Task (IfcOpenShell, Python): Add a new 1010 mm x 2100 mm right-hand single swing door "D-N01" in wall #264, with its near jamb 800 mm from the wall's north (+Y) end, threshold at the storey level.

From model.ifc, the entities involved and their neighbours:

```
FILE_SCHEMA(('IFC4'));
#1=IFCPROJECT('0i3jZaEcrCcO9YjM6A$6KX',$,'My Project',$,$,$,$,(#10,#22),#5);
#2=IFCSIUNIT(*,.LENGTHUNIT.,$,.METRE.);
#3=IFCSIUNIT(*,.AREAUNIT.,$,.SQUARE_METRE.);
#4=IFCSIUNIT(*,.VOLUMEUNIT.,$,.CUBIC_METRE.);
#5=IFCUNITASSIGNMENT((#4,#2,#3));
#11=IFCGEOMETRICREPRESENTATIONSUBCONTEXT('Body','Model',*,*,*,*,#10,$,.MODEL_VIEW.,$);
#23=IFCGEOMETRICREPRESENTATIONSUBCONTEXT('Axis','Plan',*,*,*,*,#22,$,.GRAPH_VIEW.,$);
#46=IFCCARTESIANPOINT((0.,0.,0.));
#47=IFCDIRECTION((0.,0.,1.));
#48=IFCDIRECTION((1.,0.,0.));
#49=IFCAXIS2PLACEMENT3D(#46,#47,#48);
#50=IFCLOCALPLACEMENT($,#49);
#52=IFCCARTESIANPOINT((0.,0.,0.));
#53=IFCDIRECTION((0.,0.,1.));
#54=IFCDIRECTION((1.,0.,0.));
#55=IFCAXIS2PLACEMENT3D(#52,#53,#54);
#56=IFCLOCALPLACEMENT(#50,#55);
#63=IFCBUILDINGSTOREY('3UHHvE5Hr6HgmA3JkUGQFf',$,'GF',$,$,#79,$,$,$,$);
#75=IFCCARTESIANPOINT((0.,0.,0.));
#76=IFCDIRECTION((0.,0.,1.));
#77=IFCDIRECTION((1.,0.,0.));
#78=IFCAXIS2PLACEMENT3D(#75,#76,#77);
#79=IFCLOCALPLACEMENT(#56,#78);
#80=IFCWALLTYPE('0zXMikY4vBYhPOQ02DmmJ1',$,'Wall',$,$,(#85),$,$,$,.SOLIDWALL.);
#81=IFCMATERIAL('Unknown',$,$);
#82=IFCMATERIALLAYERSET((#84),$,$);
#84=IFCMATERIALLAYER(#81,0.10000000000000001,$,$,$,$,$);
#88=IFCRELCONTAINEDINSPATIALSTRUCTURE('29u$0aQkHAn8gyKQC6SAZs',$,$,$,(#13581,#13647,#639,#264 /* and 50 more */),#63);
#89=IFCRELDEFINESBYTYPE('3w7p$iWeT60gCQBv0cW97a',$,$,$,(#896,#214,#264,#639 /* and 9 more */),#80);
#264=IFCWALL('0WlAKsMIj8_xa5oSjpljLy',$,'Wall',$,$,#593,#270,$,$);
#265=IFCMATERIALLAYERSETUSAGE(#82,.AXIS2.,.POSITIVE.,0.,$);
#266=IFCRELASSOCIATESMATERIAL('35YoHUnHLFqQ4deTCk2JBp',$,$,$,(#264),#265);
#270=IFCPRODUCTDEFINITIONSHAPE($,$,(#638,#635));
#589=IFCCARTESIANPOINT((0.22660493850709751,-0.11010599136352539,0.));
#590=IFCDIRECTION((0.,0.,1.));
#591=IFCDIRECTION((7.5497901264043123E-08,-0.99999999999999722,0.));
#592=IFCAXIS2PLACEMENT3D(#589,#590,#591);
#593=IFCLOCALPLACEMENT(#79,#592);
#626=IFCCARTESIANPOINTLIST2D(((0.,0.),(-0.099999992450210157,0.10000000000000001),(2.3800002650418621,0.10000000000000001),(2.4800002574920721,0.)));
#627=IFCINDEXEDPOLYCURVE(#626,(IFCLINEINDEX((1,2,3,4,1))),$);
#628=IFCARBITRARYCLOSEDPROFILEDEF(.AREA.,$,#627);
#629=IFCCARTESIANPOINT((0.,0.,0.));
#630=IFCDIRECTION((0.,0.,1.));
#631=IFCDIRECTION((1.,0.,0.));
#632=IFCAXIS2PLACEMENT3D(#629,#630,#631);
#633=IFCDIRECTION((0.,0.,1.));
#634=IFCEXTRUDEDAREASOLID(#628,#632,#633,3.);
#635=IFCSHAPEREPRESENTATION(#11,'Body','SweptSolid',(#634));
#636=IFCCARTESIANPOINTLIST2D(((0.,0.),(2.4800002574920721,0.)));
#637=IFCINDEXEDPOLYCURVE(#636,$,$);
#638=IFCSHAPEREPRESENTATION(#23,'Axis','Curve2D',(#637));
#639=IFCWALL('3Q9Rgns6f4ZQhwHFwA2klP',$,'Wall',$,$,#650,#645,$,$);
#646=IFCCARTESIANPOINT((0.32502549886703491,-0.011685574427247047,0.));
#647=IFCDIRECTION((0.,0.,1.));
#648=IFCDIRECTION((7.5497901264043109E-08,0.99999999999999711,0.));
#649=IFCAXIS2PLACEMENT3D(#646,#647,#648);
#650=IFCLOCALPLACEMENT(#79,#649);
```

```python
import numpy as np
import ifcopenshell
import ifcopenshell.api.feature
import ifcopenshell.api.geometry
import ifcopenshell.api.root
import ifcopenshell.api.spatial
import ifcopenshell.geom
import ifcopenshell.util.element
import ifcopenshell.util.placement
import ifcopenshell.util.representation
import ifcopenshell.util.shape
import ifcopenshell.util.unit

model = ifcopenshell.open("model.ifc")
unit_scale = ifcopenshell.util.unit.calculate_unit_scale(model)
settings = ifcopenshell.geom.settings()


def volume(element):
    """Net volume in cubic metres, openings subtracted."""
    shape = ifcopenshell.geom.create_shape(settings, element)
    return ifcopenshell.util.shape.get_volume(shape.geometry)


wall = model.by_guid("0WlAKsMIj8_xa5oSjpljLy")
storey = ifcopenshell.util.element.get_container(wall, ifc_class="IfcBuildingStorey")
context = ifcopenshell.util.representation.get_context(model, "Model", "Body", "MODEL_VIEW")
before = volume(wall)

width, height, from_end, sill = 1.01, 2.1, 0.8, 0.0  # metres

# The wall runs along its own X axis, and the end named is its -X end.
wall_shape = ifcopenshell.geom.create_shape(settings, wall)
x, y, z = ifcopenshell.util.shape.get_vertices(wall_shape.geometry).T
start = x.min() + from_end
face, thickness = float(y.min()), float(y.max() - y.min())
wall_matrix = ifcopenshell.util.placement.get_local_placement(wall.ObjectPlacement)
level = ifcopenshell.util.placement.get_local_placement(storey.ObjectPlacement)[2, 3]


def in_wall(x, y):
    """Placement at x, y metres in the wall's axes, at sill height."""
    matrix = wall_matrix.copy()
    matrix[:, 3] = wall_matrix @ np.array([x / unit_scale, y / unit_scale, 0.0, 1.0])
    matrix[2, 3] = level + sill / unit_scale
    return matrix


# Opening: a box that overshoots both wall faces by 50 mm.
opening = ifcopenshell.api.root.create_entity(model, ifc_class="IfcOpeningElement", predefined_type="OPENING")
box = ifcopenshell.api.geometry.add_wall_representation(
    model, context=context, length=width, height=height, thickness=thickness + 0.1
)
ifcopenshell.api.geometry.assign_representation(model, product=opening, representation=box)
ifcopenshell.api.geometry.edit_object_placement(model, product=opening, matrix=in_wall(start, face - 0.05), is_si=False)
ifcopenshell.api.feature.add_feature(model, feature=opening, element=wall)

door = ifcopenshell.api.root.create_entity(model, ifc_class="IfcDoor", name="D-N01", predefined_type="DOOR")
door.OverallWidth, door.OverallHeight = width / unit_scale, height / unit_scale
door.OperationType = "SINGLE_SWING_RIGHT"
body = ifcopenshell.api.geometry.add_door_representation(
    model,
    context=context,
    overall_width=door.OverallWidth,
    overall_height=door.OverallHeight,
    operation_type="SINGLE_SWING_RIGHT",
    lining_properties={"LiningDepth": thickness / unit_scale, "ThresholdDepth": thickness / unit_scale},
)
ifcopenshell.api.geometry.assign_representation(model, product=door, representation=body)
ifcopenshell.api.spatial.assign_container(model, products=[door], relating_structure=storey)
ifcopenshell.api.feature.add_filling(model, opening=opening, element=door)

# The lining spans the wall, so the door starts at the wall face.
ifcopenshell.api.geometry.edit_object_placement(model, product=door, matrix=in_wall(start, face), is_si=False)

after = volume(wall)

print(f"wall volume {before:.3f} -> {after:.3f} m3")

model.write("model-out.ifc")
```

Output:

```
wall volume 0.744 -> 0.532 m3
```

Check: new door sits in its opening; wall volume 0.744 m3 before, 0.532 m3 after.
